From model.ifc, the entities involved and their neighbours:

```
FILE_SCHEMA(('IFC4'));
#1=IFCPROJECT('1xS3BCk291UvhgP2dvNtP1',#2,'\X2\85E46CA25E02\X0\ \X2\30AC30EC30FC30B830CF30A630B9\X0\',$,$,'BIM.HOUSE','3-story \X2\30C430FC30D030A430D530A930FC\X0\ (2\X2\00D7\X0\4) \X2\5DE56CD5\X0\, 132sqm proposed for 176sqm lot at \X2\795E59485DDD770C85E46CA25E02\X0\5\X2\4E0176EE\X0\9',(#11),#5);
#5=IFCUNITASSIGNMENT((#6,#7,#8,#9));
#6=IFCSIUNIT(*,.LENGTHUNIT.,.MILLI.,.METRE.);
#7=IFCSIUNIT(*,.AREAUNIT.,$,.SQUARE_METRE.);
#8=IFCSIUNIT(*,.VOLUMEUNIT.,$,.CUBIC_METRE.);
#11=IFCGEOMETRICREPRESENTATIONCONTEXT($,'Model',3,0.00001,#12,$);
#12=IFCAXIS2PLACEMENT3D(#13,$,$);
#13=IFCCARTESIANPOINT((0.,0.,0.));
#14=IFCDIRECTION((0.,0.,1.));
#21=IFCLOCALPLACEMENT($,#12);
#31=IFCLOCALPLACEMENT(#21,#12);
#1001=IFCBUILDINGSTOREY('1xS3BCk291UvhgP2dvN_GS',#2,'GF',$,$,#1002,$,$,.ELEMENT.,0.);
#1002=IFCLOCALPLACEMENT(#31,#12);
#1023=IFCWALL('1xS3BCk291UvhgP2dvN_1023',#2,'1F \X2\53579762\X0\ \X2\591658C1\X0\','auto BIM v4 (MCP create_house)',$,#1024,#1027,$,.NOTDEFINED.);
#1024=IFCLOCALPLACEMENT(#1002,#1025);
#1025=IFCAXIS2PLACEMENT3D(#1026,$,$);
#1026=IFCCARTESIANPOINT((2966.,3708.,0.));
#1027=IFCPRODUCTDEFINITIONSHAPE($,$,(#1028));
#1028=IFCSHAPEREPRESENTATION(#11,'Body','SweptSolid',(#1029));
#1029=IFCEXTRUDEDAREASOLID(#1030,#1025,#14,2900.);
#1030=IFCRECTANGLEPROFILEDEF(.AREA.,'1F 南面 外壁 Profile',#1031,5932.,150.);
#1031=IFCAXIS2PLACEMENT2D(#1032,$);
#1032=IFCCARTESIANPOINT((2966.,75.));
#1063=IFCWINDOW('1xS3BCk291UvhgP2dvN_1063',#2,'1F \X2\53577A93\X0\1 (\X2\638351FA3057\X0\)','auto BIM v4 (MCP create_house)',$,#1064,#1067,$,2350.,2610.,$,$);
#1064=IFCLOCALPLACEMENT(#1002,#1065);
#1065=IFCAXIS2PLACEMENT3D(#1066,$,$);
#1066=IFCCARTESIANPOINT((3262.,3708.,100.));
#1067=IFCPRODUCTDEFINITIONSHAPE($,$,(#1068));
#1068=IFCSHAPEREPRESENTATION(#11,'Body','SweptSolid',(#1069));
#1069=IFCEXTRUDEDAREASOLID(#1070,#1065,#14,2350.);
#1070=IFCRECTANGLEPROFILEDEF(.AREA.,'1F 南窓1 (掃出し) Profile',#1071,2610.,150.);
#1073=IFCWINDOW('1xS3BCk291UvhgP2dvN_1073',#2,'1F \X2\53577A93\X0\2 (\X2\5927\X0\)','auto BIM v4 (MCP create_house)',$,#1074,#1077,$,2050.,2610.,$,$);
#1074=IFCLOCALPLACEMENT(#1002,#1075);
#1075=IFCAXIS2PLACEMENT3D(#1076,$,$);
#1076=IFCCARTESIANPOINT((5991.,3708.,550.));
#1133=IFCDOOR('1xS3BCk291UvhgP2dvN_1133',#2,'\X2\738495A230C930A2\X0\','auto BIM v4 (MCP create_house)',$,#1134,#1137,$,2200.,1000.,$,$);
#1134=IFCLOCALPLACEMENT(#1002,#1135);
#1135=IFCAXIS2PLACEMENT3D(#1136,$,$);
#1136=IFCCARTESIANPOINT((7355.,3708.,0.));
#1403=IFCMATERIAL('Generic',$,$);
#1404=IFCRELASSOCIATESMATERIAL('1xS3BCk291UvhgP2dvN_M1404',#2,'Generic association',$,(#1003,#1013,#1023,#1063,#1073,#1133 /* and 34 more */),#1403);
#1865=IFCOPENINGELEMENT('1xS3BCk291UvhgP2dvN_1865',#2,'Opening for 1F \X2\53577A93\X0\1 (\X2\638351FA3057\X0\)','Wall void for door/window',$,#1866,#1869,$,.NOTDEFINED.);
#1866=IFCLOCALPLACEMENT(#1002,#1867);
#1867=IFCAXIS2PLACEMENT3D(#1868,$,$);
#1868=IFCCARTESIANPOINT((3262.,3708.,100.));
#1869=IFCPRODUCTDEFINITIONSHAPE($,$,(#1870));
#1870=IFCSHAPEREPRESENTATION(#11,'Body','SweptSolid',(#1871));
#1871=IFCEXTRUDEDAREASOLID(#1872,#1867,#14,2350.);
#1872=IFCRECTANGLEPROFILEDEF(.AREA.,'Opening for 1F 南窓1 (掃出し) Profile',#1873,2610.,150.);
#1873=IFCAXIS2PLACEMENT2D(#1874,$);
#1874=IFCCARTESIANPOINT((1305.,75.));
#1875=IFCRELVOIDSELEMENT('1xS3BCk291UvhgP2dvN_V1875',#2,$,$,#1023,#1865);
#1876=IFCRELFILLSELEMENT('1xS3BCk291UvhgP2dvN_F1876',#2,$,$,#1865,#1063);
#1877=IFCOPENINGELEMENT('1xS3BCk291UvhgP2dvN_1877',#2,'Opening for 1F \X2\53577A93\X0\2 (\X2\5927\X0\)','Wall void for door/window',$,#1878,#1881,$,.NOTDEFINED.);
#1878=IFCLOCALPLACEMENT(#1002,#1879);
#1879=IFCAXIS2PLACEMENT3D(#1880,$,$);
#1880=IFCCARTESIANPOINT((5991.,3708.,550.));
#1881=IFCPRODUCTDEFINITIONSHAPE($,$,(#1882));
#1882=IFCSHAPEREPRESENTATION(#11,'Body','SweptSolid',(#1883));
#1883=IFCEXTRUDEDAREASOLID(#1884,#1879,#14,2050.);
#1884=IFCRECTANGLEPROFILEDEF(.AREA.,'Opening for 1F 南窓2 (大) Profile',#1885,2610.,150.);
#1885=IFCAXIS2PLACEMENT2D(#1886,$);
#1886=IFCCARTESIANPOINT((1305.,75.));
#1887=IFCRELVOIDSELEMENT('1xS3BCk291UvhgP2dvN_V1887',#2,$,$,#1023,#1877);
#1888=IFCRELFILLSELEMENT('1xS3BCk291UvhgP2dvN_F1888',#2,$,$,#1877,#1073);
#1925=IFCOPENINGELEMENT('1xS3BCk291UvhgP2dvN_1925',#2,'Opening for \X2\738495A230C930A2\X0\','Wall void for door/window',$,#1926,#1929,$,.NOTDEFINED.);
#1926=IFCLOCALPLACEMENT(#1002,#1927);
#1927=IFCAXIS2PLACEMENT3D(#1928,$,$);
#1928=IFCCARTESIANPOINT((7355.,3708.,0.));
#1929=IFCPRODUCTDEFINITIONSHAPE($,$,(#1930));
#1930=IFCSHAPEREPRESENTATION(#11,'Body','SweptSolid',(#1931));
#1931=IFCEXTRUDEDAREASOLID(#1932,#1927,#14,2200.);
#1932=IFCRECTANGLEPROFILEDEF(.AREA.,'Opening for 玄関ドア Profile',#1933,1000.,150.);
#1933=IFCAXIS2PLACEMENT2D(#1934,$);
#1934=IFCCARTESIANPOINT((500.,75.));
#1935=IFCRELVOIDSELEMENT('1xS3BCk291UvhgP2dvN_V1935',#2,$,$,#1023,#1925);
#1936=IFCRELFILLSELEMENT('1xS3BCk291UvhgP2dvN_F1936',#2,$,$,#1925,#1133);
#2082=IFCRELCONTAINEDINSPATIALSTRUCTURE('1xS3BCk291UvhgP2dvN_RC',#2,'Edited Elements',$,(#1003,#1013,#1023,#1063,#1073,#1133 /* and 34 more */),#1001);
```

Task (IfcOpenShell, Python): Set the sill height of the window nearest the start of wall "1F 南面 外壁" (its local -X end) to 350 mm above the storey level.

```python
import numpy as np
import ifcopenshell
import ifcopenshell.api.geometry
import ifcopenshell.geom
import ifcopenshell.util.element
import ifcopenshell.util.placement
import ifcopenshell.util.shape
import ifcopenshell.util.unit

model = ifcopenshell.open("model.ifc")
unit_scale = ifcopenshell.util.unit.calculate_unit_scale(model)

window = model.by_guid("1xS3BCk291UvhgP2dvN_1063")
opening = window.FillsVoids[0].RelatingOpeningElement
storey = ifcopenshell.util.element.get_container(window, ifc_class="IfcBuildingStorey")
level = ifcopenshell.util.placement.get_local_placement(storey.ObjectPlacement)[2, 3]

# The opening's origin need not be at the sill, so measure its lowest point.
shape = ifcopenshell.geom.create_shape(ifcopenshell.geom.settings(), opening)
bottom = ifcopenshell.util.shape.get_shape_bottom_elevation(shape, shape.geometry) / unit_scale
dz = level + 350.0 - bottom

shift = np.array([0.0, 0.0, dz])
# The window is not placed relative to its opening, so move both.
for product in (opening, window):
    matrix = ifcopenshell.util.placement.get_local_placement(product.ObjectPlacement)
    matrix[:3, 3] += shift
    ifcopenshell.api.geometry.edit_object_placement(model, product=product, matrix=matrix, is_si=False)

print(f"moved by {dz * unit_scale:+.3f} m")

model.write("model_rev.ifc")
```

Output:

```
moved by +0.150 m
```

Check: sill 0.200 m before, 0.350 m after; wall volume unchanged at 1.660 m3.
